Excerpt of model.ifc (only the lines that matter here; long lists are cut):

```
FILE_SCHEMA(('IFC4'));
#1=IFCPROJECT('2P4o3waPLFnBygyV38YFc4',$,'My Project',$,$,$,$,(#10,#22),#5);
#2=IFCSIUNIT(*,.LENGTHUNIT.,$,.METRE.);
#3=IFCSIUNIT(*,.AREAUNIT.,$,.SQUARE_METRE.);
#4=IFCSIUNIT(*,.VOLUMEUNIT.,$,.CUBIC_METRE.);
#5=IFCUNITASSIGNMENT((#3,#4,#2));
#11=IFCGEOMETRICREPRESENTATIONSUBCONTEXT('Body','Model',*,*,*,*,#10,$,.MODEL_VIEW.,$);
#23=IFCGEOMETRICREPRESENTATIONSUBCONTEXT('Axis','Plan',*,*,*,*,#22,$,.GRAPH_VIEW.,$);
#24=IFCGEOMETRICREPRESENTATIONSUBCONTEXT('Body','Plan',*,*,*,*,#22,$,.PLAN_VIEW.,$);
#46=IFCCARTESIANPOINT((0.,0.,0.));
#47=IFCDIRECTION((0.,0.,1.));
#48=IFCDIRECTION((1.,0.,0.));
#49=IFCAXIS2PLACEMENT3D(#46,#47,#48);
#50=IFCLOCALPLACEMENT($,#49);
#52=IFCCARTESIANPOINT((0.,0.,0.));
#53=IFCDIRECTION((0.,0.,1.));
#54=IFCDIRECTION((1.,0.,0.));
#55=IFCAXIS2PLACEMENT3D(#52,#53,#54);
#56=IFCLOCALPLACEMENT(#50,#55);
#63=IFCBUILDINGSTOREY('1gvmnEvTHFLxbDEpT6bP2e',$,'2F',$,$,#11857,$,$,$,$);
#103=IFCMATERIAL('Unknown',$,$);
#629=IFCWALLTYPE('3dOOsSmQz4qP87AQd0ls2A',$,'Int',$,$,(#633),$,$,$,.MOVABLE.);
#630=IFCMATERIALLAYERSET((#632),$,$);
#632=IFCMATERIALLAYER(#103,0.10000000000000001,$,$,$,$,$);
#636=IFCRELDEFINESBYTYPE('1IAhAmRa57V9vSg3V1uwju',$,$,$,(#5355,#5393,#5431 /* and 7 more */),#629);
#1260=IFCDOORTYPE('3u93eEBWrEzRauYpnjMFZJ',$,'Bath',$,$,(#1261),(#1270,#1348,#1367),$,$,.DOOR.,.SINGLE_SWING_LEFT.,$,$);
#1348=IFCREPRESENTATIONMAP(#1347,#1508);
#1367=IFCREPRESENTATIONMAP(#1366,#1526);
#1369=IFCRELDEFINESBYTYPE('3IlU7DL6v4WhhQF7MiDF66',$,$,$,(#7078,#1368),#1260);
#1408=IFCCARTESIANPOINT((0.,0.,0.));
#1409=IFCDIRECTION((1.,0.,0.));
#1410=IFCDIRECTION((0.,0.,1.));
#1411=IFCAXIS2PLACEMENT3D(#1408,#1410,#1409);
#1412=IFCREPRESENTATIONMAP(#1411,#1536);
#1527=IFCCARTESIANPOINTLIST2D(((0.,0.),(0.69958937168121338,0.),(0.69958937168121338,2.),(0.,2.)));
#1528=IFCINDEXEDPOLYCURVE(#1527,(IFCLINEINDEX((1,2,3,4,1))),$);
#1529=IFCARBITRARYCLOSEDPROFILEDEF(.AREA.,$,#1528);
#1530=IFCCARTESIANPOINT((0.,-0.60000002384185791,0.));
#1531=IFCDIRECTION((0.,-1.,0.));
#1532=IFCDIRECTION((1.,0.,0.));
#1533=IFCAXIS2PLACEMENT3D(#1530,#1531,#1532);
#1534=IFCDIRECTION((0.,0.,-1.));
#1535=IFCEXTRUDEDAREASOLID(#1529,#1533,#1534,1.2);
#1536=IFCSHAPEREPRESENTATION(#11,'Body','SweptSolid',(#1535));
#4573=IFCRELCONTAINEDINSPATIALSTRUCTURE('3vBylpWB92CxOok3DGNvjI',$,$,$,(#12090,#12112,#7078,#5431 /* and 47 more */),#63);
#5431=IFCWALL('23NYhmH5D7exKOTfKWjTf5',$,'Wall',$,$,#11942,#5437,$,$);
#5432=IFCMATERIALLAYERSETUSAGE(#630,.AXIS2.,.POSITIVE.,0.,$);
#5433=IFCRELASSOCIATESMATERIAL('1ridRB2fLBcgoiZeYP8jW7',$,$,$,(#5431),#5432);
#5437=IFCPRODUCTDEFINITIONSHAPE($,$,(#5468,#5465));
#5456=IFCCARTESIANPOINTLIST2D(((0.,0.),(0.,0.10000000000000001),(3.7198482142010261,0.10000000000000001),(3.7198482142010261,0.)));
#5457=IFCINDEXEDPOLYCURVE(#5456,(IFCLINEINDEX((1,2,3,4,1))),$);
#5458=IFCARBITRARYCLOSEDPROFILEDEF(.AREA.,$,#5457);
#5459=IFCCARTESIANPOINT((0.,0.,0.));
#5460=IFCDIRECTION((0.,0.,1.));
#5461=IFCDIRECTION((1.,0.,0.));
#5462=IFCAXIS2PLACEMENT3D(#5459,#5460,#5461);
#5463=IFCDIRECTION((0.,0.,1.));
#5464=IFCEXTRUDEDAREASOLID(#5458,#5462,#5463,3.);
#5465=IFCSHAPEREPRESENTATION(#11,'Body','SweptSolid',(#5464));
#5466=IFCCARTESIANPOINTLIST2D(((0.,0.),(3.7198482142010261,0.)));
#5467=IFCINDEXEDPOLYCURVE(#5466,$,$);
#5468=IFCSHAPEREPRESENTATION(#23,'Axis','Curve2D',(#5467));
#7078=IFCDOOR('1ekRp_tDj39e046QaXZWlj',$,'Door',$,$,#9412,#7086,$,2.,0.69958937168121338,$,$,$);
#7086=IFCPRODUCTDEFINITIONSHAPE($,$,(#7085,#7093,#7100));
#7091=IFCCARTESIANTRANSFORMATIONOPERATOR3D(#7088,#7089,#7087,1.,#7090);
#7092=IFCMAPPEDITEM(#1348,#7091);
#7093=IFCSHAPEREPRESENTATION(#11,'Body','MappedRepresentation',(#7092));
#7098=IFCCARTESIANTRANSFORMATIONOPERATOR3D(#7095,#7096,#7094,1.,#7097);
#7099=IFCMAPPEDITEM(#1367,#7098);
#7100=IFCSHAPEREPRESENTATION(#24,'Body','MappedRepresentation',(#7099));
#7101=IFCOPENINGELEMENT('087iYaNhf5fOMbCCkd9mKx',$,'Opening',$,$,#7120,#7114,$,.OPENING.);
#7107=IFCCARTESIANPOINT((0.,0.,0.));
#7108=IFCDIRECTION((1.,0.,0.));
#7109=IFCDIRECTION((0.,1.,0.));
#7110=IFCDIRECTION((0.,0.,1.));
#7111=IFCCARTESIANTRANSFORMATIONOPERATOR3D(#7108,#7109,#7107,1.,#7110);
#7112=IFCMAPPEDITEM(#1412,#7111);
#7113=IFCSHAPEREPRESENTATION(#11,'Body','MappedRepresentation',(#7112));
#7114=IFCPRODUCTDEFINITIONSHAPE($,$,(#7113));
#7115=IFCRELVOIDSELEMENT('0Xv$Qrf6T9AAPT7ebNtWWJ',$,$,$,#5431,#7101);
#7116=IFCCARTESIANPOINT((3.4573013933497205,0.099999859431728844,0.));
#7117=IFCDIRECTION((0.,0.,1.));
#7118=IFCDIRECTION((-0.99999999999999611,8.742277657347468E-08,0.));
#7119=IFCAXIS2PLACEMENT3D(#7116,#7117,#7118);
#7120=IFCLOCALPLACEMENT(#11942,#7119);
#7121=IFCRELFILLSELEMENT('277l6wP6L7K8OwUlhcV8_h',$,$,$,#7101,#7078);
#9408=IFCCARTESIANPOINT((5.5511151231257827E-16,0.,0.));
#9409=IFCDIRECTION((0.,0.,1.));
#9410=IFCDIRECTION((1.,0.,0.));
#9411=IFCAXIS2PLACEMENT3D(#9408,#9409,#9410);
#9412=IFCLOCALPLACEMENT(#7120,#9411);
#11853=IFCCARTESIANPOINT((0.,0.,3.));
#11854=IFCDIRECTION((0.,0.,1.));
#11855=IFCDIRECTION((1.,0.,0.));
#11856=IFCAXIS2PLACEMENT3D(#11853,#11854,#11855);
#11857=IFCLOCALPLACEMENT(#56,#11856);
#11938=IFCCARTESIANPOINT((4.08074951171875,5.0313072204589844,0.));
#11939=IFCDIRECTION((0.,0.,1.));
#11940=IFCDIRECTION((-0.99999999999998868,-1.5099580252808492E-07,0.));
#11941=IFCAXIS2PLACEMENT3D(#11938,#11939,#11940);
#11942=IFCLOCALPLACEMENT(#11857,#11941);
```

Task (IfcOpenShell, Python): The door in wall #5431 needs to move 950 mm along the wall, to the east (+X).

```python
import ifcopenshell
import ifcopenshell.api.geometry
import ifcopenshell.util.placement

model = ifcopenshell.open("model.ifc")

door = model.by_guid("1ekRp_tDj39e046QaXZWlj")
opening = door.FillsVoids[0].RelatingOpeningElement
wall = opening.VoidsElements[0].RelatingBuildingElement

wall_matrix = ifcopenshell.util.placement.get_local_placement(wall.ObjectPlacement)
shift = wall_matrix[:3, 0] * -0.95
before = ifcopenshell.util.placement.get_local_placement(door.ObjectPlacement)[:3, 3].copy()

# The door is placed relative to its opening, so it follows when the opening moves.
matrix = ifcopenshell.util.placement.get_local_placement(opening.ObjectPlacement)
matrix[:3, 3] += shift
ifcopenshell.api.geometry.edit_object_placement(
    model, product=opening, matrix=matrix, is_si=False, should_transform_children=True
)

after = ifcopenshell.util.placement.get_local_placement(door.ObjectPlacement)[:3, 3]
print("door moved by", (after - before).round(3) + 0.0)

model.write("model_rev.ifc")
```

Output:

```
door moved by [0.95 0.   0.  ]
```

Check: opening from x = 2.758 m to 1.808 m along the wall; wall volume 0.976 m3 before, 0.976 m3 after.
